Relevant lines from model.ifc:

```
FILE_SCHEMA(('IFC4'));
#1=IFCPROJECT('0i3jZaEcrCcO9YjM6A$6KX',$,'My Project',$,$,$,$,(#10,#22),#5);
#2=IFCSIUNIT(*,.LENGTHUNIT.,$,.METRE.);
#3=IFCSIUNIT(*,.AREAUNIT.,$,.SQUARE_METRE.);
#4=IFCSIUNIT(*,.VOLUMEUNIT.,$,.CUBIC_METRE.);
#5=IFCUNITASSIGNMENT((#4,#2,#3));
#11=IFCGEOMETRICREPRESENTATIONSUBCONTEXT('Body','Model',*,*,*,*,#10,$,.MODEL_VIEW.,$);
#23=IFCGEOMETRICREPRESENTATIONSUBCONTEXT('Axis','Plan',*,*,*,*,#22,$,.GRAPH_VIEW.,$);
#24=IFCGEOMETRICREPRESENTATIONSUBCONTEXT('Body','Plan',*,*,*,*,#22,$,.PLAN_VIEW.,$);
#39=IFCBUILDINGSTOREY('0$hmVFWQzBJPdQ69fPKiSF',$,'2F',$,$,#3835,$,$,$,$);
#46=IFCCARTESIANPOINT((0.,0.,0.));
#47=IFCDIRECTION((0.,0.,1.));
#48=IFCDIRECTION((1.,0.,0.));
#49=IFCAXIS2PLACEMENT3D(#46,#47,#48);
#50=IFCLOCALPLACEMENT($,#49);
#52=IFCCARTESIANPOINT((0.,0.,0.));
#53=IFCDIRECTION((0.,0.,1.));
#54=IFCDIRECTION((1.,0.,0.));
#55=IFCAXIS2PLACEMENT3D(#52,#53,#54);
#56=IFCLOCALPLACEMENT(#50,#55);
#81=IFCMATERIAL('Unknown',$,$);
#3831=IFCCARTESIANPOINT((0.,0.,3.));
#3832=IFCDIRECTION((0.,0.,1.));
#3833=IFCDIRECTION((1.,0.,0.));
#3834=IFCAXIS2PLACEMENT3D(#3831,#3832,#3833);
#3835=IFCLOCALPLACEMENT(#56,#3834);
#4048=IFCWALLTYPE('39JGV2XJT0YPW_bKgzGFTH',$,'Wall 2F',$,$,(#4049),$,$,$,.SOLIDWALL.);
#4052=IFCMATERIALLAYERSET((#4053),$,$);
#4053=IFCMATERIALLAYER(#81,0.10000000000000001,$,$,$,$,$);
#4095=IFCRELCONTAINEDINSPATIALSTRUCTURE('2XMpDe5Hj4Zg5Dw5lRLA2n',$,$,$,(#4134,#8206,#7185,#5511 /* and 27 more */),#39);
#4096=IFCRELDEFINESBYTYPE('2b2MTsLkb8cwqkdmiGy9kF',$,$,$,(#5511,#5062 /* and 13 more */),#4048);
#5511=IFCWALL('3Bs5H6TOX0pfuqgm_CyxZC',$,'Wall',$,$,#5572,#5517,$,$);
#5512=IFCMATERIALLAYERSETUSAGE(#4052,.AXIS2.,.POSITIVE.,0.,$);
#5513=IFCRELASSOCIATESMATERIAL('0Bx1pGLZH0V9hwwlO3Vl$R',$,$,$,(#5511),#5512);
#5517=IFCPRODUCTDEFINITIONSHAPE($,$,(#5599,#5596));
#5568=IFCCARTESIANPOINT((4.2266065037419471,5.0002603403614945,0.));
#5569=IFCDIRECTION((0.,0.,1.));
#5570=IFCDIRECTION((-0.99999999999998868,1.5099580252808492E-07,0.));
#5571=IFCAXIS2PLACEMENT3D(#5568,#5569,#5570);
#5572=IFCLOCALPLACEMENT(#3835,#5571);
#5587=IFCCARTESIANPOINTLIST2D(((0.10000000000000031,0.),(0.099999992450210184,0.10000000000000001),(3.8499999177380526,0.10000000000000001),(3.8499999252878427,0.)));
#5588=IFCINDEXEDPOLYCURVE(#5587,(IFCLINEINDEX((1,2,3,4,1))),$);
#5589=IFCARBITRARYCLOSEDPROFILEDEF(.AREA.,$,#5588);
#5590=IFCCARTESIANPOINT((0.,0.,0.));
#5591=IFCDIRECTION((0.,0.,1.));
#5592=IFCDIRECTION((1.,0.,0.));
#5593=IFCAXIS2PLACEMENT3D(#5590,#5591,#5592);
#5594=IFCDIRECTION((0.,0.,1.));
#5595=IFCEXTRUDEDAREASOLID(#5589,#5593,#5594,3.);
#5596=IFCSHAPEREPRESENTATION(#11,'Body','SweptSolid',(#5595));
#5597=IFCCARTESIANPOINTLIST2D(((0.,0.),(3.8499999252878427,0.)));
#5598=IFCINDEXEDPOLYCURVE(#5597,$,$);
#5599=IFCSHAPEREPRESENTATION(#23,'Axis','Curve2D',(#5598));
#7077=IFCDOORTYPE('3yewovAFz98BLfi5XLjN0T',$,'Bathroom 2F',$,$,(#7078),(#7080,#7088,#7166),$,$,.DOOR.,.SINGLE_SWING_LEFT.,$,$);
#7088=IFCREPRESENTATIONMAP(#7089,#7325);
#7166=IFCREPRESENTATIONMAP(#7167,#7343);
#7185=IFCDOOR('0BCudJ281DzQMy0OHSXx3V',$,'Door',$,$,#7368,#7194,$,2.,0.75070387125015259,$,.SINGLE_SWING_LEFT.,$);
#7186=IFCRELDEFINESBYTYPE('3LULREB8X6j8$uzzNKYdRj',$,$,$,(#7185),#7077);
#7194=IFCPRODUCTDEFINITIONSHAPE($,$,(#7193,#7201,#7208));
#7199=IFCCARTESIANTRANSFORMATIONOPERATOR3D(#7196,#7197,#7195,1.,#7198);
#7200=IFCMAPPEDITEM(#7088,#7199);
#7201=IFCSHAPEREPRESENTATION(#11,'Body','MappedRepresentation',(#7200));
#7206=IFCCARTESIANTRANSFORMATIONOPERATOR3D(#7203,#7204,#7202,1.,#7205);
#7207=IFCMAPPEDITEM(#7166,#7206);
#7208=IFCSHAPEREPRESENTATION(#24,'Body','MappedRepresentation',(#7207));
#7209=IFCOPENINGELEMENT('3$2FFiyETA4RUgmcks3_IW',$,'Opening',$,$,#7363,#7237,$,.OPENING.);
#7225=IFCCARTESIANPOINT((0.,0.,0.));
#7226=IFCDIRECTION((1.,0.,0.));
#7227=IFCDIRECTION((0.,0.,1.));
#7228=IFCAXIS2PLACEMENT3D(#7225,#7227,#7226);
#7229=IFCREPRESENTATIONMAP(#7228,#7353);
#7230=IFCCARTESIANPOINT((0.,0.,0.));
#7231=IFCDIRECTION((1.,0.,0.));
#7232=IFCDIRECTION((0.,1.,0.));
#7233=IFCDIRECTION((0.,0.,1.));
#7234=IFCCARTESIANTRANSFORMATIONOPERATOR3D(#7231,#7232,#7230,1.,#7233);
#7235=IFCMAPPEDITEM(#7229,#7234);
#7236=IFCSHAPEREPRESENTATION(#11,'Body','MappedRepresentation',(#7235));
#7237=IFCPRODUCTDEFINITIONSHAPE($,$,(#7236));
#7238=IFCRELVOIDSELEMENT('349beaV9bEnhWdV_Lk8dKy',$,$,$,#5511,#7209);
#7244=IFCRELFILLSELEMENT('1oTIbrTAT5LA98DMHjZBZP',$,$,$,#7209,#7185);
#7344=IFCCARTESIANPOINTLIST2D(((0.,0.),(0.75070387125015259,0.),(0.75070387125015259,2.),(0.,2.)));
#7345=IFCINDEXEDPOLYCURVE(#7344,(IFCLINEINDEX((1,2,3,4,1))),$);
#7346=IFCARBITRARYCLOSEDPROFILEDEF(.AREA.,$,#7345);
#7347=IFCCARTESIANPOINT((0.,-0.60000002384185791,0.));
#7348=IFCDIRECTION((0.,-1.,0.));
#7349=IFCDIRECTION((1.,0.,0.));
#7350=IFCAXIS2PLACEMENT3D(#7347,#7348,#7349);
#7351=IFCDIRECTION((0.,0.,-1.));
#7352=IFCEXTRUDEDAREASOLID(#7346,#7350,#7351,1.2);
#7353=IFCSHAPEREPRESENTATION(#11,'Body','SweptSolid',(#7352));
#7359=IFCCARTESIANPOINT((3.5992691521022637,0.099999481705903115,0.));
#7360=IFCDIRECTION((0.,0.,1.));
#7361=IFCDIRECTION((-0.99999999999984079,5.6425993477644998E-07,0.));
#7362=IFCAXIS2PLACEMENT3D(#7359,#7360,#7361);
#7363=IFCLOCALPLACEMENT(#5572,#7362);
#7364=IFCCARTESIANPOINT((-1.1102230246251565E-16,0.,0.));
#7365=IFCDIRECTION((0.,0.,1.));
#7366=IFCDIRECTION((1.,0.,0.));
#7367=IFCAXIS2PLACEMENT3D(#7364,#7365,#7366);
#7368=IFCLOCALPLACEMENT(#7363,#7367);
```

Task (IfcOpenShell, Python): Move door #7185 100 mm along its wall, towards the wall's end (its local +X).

```python
import ifcopenshell
import ifcopenshell.api.geometry
import ifcopenshell.util.placement
import ifcopenshell.util.unit

model = ifcopenshell.open("model.ifc")
unit_scale = ifcopenshell.util.unit.calculate_unit_scale(model)

door = model.by_guid("0BCudJ281DzQMy0OHSXx3V")
opening = door.FillsVoids[0].RelatingOpeningElement
wall = opening.VoidsElements[0].RelatingBuildingElement

wall_matrix = ifcopenshell.util.placement.get_local_placement(wall.ObjectPlacement)
shift = wall_matrix[:3, 0] * 0.1 / unit_scale
before = ifcopenshell.util.placement.get_local_placement(door.ObjectPlacement)[:3, 3].copy()

# The door is placed relative to its opening, so it follows when the opening moves.
matrix = ifcopenshell.util.placement.get_local_placement(opening.ObjectPlacement)
matrix[:3, 3] += shift
ifcopenshell.api.geometry.edit_object_placement(
    model, product=opening, matrix=matrix, is_si=False, should_transform_children=True
)

after = ifcopenshell.util.placement.get_local_placement(door.ObjectPlacement)[:3, 3]
print("door moved by", (after - before).round(3) + 0.0)

model.write("model_rev.ifc")
```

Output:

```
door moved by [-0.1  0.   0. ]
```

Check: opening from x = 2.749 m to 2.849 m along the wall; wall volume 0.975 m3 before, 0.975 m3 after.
